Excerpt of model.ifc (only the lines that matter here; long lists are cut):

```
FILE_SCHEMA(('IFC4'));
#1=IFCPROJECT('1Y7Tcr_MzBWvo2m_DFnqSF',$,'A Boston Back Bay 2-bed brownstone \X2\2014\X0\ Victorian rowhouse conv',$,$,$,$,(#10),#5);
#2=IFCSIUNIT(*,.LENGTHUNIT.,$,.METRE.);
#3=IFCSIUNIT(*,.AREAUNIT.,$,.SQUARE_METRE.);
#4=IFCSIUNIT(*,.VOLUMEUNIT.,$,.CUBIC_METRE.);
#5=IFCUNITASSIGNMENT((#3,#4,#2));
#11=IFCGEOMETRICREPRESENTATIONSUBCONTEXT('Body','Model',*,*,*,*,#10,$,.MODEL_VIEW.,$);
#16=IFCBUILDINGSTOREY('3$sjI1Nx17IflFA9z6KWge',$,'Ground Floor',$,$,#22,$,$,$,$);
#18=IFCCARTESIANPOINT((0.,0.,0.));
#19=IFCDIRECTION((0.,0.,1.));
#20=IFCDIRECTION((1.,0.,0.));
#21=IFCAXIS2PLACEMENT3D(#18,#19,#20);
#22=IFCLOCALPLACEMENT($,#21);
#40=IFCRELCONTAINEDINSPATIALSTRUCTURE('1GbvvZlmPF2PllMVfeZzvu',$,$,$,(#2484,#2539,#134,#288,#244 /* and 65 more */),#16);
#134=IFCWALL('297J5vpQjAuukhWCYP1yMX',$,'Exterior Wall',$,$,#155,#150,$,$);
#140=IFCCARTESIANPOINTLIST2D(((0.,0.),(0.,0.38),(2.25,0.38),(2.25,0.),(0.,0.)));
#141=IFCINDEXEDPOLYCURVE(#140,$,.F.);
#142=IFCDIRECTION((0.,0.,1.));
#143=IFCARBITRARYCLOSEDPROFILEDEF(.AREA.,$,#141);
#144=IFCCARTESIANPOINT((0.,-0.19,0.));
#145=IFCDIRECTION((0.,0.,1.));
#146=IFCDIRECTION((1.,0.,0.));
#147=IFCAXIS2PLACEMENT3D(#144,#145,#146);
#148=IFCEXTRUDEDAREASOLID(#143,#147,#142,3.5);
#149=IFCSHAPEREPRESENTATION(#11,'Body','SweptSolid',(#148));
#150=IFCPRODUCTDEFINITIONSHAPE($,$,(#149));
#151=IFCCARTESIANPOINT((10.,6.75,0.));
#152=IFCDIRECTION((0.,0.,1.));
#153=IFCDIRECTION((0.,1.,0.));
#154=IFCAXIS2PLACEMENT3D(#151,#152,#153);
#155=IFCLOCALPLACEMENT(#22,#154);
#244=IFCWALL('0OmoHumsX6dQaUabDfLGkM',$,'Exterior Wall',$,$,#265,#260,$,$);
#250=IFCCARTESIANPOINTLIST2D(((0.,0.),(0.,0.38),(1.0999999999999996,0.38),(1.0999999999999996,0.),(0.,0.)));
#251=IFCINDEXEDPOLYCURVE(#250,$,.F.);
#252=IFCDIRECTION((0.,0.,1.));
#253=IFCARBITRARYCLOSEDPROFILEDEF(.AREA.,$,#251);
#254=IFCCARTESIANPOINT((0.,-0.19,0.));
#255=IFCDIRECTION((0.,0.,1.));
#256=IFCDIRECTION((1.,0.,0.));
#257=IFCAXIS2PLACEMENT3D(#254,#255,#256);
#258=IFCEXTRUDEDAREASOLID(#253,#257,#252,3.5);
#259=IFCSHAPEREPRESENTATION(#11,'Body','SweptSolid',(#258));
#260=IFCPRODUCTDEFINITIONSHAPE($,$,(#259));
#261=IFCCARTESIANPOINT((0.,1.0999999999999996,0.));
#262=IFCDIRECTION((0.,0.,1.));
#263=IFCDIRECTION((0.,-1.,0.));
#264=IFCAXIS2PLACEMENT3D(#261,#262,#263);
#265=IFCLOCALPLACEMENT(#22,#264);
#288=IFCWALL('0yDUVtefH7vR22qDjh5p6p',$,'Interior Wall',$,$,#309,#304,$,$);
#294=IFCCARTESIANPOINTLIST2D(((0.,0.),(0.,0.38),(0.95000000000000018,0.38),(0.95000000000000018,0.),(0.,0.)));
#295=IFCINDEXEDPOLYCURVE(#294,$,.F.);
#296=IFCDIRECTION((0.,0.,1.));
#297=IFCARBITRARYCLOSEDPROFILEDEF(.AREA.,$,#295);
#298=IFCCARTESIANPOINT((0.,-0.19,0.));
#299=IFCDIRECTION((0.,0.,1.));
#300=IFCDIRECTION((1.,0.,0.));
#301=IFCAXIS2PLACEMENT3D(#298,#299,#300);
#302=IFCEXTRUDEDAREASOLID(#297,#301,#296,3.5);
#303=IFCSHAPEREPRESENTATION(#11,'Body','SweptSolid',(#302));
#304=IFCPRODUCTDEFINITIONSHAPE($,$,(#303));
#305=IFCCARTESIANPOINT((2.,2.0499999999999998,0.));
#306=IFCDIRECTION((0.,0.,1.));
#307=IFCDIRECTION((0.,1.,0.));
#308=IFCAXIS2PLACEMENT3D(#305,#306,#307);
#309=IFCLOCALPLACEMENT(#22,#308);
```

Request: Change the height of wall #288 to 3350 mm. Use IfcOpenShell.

```python
import ifcopenshell
import ifcopenshell.geom
import ifcopenshell.util.representation
import ifcopenshell.util.shape
import ifcopenshell.util.unit

model = ifcopenshell.open("model.ifc")
unit_scale = ifcopenshell.util.unit.calculate_unit_scale(model)
settings = ifcopenshell.geom.settings()


def volume(element):
    """Net volume in cubic metres, openings subtracted."""
    shape = ifcopenshell.geom.create_shape(settings, element)
    return ifcopenshell.util.shape.get_volume(shape.geometry)


wall = model.by_guid("0yDUVtefH7vR22qDjh5p6p")
before = volume(wall)

body = ifcopenshell.util.representation.get_representation(wall, "Model", "Body")
solid = body.Items[0]
old_height = solid.Depth
solid.Depth = 3.35 / unit_scale
after = volume(wall)

print(f"height {old_height:g} -> {solid.Depth:g}, volume {before:.3f} -> {after:.3f} m3")

model.write("model_v2.ifc")
```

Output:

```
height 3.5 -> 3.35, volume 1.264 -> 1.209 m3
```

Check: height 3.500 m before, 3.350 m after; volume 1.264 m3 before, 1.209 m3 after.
